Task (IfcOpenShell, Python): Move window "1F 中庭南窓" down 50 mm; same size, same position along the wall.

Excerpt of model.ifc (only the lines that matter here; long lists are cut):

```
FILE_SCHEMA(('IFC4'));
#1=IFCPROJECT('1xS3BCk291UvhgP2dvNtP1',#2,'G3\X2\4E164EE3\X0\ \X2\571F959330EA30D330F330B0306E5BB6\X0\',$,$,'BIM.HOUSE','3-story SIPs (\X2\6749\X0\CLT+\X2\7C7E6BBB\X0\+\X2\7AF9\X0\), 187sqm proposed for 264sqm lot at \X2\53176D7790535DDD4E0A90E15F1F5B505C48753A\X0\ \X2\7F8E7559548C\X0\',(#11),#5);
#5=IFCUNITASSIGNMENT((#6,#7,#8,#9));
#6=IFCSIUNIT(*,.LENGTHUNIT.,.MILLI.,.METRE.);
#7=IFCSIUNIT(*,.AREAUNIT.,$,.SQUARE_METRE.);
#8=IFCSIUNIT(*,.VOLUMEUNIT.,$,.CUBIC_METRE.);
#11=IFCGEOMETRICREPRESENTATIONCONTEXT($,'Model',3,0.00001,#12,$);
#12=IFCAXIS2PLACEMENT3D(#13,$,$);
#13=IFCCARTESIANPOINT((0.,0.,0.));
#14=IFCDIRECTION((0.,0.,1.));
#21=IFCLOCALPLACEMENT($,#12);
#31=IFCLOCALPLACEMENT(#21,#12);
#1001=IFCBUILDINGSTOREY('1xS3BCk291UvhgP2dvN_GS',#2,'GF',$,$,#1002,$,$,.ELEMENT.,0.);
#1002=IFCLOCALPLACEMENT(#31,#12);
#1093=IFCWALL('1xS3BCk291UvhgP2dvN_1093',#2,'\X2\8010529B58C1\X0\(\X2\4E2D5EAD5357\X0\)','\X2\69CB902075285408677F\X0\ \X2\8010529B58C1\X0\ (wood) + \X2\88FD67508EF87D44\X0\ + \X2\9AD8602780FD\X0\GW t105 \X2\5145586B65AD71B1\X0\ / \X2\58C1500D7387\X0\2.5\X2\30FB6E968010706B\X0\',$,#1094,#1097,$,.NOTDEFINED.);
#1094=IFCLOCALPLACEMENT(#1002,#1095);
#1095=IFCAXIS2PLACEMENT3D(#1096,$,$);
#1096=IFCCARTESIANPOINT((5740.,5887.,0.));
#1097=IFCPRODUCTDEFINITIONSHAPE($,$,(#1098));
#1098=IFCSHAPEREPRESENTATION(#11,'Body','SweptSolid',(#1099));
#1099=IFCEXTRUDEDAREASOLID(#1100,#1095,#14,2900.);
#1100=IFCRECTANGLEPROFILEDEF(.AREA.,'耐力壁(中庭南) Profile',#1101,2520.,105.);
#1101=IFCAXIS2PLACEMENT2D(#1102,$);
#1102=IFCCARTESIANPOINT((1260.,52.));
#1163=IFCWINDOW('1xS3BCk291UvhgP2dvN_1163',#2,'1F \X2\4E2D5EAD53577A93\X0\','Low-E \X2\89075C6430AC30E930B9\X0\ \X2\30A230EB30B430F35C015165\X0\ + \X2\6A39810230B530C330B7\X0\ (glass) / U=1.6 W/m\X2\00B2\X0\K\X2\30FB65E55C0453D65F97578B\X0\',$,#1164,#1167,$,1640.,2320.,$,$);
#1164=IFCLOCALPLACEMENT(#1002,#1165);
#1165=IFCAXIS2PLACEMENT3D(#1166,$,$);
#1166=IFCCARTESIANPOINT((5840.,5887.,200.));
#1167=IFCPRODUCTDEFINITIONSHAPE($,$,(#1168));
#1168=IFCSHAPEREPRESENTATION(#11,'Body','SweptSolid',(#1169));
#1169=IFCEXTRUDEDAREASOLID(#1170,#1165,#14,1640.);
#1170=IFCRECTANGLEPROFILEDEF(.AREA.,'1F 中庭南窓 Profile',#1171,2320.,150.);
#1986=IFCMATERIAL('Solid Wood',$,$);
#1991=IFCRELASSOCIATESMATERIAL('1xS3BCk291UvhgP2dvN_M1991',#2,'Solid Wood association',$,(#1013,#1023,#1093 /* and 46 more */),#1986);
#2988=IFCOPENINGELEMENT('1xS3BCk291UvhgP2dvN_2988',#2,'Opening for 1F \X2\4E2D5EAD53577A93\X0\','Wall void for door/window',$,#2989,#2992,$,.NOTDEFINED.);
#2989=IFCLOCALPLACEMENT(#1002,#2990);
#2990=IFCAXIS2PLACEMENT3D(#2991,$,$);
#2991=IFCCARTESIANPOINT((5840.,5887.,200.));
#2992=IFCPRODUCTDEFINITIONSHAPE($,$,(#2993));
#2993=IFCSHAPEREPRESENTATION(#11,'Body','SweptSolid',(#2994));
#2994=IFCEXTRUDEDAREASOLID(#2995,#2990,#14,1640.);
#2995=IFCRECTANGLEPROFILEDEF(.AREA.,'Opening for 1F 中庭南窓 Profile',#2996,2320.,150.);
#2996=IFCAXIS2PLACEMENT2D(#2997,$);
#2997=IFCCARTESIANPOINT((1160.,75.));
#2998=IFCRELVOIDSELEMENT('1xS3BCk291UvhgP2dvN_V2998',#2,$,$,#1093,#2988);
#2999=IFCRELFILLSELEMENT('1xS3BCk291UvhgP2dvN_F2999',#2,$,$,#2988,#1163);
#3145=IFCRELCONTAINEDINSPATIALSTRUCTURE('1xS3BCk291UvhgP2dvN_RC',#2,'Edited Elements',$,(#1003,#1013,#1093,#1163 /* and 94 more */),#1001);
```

```python
import numpy as np
import ifcopenshell
import ifcopenshell.api.geometry
import ifcopenshell.util.placement
import ifcopenshell.util.unit

model = ifcopenshell.open("model.ifc")
unit_scale = ifcopenshell.util.unit.calculate_unit_scale(model)

window = model.by_id(1163)
opening = window.FillsVoids[0].RelatingOpeningElement
dz = -0.05 / unit_scale

shift = np.array([0.0, 0.0, dz])
# The window is not placed relative to its opening, so move both.
for product in (opening, window):
    matrix = ifcopenshell.util.placement.get_local_placement(product.ObjectPlacement)
    matrix[:3, 3] += shift
    ifcopenshell.api.geometry.edit_object_placement(model, product=product, matrix=matrix, is_si=False)

print(f"moved by {dz * unit_scale:+.3f} m")

model.write("model_v2.ifc")
```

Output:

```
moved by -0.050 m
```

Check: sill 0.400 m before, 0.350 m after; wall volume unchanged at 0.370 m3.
